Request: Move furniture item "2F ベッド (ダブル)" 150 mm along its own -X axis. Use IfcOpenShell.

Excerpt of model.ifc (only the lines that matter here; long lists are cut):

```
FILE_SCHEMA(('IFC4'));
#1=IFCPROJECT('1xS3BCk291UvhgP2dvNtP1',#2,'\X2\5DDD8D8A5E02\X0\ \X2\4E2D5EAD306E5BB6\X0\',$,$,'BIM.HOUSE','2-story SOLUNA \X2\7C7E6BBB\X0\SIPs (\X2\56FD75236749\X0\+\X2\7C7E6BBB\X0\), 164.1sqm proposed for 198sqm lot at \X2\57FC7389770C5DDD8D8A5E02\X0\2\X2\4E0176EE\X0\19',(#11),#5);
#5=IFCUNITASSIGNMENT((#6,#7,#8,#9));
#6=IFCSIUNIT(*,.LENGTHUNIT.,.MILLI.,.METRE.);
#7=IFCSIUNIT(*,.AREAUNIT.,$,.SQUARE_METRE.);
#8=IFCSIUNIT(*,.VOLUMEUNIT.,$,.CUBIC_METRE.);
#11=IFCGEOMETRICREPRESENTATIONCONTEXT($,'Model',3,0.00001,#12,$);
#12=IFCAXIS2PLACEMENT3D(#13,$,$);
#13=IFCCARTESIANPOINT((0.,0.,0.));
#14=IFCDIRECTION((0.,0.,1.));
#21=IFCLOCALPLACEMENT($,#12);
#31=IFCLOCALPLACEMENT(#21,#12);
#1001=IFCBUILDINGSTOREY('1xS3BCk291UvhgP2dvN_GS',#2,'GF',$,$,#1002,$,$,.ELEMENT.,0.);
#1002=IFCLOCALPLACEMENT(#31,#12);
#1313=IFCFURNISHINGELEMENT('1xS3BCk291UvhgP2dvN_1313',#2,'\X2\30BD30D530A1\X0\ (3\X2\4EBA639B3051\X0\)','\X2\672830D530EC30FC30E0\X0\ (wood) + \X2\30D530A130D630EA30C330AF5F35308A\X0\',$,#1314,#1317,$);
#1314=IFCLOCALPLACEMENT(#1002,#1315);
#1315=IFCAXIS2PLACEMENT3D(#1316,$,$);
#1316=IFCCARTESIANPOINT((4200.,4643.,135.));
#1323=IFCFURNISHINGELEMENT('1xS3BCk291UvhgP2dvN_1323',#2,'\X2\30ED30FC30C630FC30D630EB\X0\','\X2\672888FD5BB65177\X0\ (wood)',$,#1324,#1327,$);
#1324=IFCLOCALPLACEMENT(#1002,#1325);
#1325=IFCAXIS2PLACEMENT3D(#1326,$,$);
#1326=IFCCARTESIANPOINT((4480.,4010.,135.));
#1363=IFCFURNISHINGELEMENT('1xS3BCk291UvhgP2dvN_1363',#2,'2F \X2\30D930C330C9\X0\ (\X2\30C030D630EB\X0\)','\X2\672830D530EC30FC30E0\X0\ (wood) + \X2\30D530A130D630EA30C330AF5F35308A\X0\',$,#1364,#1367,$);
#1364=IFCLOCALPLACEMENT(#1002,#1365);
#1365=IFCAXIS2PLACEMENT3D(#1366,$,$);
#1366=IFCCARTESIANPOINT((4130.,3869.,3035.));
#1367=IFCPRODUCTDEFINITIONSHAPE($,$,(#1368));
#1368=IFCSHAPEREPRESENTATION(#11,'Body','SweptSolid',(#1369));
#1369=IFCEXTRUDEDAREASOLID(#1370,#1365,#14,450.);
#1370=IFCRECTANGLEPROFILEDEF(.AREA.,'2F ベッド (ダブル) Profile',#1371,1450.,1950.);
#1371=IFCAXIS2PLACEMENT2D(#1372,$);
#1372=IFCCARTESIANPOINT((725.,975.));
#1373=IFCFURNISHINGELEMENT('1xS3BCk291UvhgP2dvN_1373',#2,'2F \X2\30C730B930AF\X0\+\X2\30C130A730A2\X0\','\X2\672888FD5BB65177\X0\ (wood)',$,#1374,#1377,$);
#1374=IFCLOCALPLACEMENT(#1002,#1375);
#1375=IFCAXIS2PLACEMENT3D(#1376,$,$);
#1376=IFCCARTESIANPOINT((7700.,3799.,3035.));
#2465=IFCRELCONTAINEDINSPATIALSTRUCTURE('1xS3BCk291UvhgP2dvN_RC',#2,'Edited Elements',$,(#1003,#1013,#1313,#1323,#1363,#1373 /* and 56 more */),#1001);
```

```python
import ifcopenshell
import ifcopenshell.api.geometry
import ifcopenshell.util.placement
import ifcopenshell.util.unit

model = ifcopenshell.open("model.ifc")
unit_scale = ifcopenshell.util.unit.calculate_unit_scale(model)

item = model.by_guid("1xS3BCk291UvhgP2dvN_1363")
matrix = ifcopenshell.util.placement.get_local_placement(item.ObjectPlacement)
matrix[:3, 3] -= matrix[:3, 0] * 0.15 / unit_scale
ifcopenshell.api.geometry.edit_object_placement(model, product=item, matrix=matrix, is_si=False)

print(ifcopenshell.util.placement.get_local_placement(item.ObjectPlacement).round(3) + 0.0)

model.write("model_rev.ifc")
```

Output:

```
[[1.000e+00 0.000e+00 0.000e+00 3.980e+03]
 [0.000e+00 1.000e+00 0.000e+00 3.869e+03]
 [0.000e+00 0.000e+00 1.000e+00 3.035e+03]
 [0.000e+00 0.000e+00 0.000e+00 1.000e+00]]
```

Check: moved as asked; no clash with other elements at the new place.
